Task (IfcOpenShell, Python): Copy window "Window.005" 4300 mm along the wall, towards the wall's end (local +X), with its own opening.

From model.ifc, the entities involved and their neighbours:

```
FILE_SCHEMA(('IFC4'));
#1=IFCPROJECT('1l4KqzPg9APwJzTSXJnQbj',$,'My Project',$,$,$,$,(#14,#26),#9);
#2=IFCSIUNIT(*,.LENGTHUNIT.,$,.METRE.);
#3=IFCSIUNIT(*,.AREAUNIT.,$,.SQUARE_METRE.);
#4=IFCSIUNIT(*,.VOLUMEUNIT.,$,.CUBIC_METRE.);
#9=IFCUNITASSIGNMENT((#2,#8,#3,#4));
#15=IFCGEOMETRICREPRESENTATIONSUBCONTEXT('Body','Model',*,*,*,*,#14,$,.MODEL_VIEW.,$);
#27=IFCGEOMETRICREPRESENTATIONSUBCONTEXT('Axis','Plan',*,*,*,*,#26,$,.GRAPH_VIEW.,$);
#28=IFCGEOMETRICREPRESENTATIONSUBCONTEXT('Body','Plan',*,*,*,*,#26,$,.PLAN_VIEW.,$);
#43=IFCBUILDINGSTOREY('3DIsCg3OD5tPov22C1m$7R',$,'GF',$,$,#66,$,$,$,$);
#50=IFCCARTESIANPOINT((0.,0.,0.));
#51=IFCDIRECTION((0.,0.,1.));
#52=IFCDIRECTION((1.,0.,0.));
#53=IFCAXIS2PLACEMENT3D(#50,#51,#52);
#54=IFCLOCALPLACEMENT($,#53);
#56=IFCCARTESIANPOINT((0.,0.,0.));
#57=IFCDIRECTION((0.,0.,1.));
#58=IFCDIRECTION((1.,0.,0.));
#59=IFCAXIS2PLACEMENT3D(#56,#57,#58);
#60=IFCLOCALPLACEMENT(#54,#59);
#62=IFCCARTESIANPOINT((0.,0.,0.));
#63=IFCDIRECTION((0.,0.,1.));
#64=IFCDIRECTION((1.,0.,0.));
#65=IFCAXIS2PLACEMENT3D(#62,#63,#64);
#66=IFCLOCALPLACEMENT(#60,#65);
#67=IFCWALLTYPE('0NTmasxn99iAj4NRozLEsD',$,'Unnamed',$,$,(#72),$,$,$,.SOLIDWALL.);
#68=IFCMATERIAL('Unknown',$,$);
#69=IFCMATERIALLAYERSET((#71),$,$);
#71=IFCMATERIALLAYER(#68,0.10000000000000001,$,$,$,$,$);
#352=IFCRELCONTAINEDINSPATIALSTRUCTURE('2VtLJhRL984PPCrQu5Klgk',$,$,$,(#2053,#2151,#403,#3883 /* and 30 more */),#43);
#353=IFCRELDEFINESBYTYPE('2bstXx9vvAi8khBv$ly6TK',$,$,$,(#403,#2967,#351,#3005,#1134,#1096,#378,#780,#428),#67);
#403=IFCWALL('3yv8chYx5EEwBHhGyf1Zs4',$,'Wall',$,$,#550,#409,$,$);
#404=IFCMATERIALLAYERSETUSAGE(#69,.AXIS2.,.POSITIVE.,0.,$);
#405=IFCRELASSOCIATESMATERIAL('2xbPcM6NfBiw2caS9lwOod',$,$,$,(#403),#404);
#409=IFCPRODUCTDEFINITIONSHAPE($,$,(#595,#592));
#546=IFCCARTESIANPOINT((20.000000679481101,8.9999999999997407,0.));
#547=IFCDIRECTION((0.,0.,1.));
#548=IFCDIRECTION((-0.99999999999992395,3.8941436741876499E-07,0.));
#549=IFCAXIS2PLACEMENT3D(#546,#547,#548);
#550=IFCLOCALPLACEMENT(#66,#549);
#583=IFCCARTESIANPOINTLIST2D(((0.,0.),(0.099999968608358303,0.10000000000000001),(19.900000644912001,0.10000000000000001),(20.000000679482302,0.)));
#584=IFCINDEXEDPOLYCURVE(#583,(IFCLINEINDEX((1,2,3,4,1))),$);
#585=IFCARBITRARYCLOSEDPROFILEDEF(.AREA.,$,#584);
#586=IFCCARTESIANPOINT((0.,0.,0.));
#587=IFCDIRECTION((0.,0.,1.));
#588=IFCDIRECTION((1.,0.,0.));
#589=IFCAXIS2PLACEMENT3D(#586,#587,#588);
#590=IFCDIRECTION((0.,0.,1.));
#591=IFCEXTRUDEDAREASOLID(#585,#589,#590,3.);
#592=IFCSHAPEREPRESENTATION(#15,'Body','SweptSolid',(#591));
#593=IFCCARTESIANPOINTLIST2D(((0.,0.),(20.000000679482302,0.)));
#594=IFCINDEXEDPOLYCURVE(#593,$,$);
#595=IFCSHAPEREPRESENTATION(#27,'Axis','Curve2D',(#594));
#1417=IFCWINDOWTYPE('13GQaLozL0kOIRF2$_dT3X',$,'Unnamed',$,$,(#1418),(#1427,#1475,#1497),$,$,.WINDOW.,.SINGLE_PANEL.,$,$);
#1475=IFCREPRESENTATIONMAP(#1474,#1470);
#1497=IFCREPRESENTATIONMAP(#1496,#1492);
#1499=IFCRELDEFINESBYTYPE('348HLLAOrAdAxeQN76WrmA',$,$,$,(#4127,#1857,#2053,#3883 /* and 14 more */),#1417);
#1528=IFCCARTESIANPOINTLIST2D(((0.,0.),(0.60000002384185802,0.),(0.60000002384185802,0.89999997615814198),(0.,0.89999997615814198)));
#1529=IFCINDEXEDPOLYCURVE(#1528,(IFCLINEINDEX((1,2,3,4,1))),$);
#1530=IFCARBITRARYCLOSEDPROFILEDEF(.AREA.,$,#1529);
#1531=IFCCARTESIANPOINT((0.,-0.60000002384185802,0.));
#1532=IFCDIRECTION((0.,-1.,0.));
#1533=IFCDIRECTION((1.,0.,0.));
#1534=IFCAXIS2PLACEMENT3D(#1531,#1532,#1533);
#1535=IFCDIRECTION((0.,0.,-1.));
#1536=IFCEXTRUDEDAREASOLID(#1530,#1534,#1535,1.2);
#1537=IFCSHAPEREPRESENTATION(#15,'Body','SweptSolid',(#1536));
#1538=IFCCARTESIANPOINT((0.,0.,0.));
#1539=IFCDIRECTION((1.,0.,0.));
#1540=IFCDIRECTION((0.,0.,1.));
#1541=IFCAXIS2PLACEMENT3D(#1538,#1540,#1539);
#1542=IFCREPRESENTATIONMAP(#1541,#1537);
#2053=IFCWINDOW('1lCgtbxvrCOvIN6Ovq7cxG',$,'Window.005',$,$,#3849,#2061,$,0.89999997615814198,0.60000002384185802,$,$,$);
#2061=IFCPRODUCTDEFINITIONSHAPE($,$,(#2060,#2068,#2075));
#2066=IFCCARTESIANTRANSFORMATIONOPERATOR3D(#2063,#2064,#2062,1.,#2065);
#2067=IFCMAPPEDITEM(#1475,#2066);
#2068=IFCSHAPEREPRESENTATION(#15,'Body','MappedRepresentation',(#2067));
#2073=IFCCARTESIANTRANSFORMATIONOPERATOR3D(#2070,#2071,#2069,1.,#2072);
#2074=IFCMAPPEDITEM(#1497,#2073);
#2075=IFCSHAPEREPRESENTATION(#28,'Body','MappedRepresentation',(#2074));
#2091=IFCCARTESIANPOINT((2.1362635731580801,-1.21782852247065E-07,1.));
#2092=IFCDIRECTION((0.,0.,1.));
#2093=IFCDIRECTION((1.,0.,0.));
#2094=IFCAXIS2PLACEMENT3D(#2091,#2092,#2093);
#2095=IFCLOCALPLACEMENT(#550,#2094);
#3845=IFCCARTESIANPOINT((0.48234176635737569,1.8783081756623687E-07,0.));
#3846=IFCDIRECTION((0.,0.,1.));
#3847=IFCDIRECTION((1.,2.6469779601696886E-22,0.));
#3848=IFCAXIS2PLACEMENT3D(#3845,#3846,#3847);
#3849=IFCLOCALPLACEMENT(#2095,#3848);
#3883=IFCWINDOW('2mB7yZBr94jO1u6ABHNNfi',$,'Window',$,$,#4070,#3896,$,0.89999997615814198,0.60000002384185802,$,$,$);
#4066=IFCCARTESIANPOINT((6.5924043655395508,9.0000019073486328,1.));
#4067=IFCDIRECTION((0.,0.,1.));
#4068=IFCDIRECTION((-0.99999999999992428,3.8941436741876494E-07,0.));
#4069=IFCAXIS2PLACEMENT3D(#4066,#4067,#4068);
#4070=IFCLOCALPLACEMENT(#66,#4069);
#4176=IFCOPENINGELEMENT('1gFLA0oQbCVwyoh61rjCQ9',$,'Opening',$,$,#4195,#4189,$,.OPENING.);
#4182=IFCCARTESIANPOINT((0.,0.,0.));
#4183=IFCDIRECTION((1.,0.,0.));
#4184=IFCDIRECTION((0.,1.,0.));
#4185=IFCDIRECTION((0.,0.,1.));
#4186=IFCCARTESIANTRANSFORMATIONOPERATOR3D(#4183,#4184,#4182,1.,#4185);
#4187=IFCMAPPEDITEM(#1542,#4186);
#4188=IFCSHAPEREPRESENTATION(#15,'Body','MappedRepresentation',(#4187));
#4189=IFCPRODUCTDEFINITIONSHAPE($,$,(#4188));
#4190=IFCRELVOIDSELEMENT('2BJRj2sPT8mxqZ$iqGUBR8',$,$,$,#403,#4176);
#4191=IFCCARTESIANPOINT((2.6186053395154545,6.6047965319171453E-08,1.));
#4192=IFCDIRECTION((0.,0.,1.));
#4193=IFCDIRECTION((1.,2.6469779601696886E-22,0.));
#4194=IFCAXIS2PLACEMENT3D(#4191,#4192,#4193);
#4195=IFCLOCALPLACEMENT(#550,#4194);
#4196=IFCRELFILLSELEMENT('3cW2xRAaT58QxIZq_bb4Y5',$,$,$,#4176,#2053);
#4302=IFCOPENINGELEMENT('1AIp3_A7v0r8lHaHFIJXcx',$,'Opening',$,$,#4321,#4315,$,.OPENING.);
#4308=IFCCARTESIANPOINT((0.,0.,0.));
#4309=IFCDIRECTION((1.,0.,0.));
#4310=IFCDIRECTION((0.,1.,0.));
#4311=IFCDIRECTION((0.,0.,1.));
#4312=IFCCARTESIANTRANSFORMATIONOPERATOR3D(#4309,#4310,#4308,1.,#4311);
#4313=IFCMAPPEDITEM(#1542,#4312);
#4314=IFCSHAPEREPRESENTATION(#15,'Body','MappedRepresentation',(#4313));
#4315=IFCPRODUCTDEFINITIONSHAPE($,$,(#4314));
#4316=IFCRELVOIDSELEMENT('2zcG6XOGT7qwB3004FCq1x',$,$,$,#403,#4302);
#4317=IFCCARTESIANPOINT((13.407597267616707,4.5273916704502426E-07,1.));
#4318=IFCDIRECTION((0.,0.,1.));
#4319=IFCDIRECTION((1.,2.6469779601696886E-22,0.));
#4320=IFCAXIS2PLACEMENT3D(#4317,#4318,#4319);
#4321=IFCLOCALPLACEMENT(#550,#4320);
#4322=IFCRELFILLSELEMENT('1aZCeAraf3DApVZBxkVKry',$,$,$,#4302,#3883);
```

```python
import ifcopenshell
import ifcopenshell.api.feature
import ifcopenshell.api.geometry
import ifcopenshell.api.root
import ifcopenshell.geom
import ifcopenshell.util.element
import ifcopenshell.util.placement
import ifcopenshell.util.shape
import ifcopenshell.util.unit

model = ifcopenshell.open("model.ifc")
unit_scale = ifcopenshell.util.unit.calculate_unit_scale(model)
settings = ifcopenshell.geom.settings()


def volume(element):
    """Net volume in cubic metres, openings subtracted."""
    shape = ifcopenshell.geom.create_shape(settings, element)
    return ifcopenshell.util.shape.get_volume(shape.geometry)


window = model.by_guid("1lCgtbxvrCOvIN6Ovq7cxG")
opening = window.FillsVoids[0].RelatingOpeningElement
wall = opening.VoidsElements[0].RelatingBuildingElement
before = volume(wall)
shift = ifcopenshell.util.placement.get_local_placement(wall.ObjectPlacement)[:3, 0] * 4.3 / unit_scale

# copy_class copies the void relationship, type, container and properties, but no geometry.
new_opening = ifcopenshell.api.root.copy_class(model, product=opening)
new_opening.Representation = ifcopenshell.util.element.copy_deep(
    model, opening.Representation, exclude=["IfcGeometricRepresentationContext", "IfcRepresentationMap"]
)
new_window = ifcopenshell.api.root.copy_class(model, product=window)
new_window.Representation = ifcopenshell.util.element.copy_deep(
    model, window.Representation, exclude=["IfcGeometricRepresentationContext", "IfcRepresentationMap"]
)
ifcopenshell.api.feature.add_filling(model, opening=new_opening, element=new_window)

for old, new in ((opening, new_opening), (window, new_window)):
    matrix = ifcopenshell.util.placement.get_local_placement(old.ObjectPlacement)
    matrix[:3, 3] += shift
    ifcopenshell.api.geometry.edit_object_placement(model, product=new, matrix=matrix, is_si=False)

after = volume(wall)

print(f"wall volume {before:.3f} -> {after:.3f} m3")

model.write("model_v2.ifc")
```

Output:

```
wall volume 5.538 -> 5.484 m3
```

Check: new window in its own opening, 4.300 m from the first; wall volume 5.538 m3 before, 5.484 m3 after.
